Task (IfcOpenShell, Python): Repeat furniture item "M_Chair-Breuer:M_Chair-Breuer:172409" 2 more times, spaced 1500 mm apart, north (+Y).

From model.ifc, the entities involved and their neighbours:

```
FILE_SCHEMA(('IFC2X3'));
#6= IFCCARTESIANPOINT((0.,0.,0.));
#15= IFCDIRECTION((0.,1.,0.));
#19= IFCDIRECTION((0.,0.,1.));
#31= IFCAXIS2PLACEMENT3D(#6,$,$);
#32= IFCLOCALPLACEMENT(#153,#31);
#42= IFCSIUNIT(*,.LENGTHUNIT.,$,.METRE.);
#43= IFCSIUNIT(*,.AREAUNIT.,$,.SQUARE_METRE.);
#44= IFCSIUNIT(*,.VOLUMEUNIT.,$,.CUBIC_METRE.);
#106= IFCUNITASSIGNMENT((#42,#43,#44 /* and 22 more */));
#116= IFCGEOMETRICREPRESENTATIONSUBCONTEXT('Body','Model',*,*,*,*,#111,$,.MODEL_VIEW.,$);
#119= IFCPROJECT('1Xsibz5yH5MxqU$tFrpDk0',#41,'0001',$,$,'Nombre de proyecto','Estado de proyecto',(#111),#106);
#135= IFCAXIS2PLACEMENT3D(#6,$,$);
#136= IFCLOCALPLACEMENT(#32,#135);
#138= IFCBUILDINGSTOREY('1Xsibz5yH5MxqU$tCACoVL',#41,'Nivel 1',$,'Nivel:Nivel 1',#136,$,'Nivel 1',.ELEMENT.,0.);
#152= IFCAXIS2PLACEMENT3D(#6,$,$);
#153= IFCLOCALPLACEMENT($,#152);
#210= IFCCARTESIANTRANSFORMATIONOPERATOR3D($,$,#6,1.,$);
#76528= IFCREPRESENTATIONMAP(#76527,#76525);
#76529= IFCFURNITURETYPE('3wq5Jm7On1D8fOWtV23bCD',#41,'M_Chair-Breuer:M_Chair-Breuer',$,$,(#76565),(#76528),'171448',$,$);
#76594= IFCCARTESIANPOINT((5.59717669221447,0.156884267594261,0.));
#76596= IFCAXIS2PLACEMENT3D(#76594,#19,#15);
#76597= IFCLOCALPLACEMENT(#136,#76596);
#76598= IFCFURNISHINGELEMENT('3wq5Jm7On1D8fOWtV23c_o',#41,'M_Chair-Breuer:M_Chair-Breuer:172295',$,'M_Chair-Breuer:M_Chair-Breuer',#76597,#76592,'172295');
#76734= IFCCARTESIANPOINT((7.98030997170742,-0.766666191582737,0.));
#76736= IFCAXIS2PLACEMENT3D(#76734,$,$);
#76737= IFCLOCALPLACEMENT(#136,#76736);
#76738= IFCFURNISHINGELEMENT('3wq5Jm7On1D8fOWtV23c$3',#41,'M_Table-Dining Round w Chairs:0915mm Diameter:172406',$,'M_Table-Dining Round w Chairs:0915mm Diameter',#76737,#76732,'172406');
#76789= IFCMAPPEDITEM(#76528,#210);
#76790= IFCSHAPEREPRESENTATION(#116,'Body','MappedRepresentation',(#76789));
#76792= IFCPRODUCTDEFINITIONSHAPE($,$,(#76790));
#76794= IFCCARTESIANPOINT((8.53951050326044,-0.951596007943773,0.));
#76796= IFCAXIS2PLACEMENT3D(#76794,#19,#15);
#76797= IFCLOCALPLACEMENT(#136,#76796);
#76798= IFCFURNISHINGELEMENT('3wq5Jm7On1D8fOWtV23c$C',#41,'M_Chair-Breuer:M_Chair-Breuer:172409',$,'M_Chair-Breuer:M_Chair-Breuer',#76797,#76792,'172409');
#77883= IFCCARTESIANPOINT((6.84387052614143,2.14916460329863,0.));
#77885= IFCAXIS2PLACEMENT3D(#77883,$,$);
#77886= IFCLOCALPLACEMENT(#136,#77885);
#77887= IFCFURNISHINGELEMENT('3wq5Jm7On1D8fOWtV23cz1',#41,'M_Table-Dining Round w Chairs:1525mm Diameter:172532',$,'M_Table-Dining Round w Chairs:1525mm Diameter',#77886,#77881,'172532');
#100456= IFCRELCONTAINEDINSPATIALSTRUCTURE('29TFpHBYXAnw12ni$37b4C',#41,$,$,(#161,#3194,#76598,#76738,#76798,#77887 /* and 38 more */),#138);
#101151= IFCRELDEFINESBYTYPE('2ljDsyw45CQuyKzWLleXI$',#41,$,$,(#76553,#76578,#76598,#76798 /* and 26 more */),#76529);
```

```python
import numpy as np
import ifcopenshell
import ifcopenshell.api.geometry
import ifcopenshell.api.root
import ifcopenshell.util.element
import ifcopenshell.util.placement
import ifcopenshell.util.unit

model = ifcopenshell.open("model.ifc")
unit_scale = ifcopenshell.util.unit.calculate_unit_scale(model)


def reuse_history(source, copy):
    """copy_class also copies each property set's owner history, people and application; keep the originals."""
    for rel in copy.IsDefinedBy:
        if rel.is_a("IfcRelDefinesByProperties") and (history := rel.RelatingPropertyDefinition.OwnerHistory):
            rel.RelatingPropertyDefinition.OwnerHistory = source.OwnerHistory
            ifcopenshell.util.element.remove_deep2(model, history)


source = model.by_guid("3wq5Jm7On1D8fOWtV23c$C")
base = ifcopenshell.util.placement.get_local_placement(source.ObjectPlacement)
step = np.array([0.0, 1.0, 0.0]) * 1.5 / unit_scale

for i in range(1, 3):
    copy = ifcopenshell.api.root.copy_class(model, product=source)
    copy.Representation = ifcopenshell.util.element.copy_deep(
        model, source.Representation, exclude=["IfcGeometricRepresentationContext", "IfcRepresentationMap"]
    )
    copy.Name = "M_Chair-Breuer:M_Chair-Breuer"
    copy.Tag = None
    reuse_history(source, copy)
    matrix = base.copy()
    matrix[:3, 3] += i * step
    print("added at", matrix[:3, 3].round(3) + 0.0)
    ifcopenshell.api.geometry.edit_object_placement(model, product=copy, matrix=matrix, is_si=False)

model.write("model_rev.ifc")
```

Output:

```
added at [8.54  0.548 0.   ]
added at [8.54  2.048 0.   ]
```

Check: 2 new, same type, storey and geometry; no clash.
